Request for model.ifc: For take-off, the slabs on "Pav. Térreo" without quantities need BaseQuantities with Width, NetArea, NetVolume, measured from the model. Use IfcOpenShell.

First a look at what the model holds.

```python
import ifcopenshell
import ifcopenshell.util.element
import ifcopenshell.util.unit

model = ifcopenshell.open("model.ifc")
print(model.schema)
for unit_type in ("LENGTHUNIT", "AREAUNIT", "VOLUMEUNIT"):
    print(unit_type, ifcopenshell.util.unit.calculate_unit_scale(model, unit_type))
storey = next(s for s in model.by_type("IfcBuildingStorey") if s.Name == "Pav. Térreo")
slabs = [e for e in ifcopenshell.util.element.get_decomposition(storey) if e.is_a("IfcSlab")]
for e in sorted(slabs, key=lambda e: e.id()):
    print(e.id(), e.is_a(), e.Name, list(ifcopenshell.util.element.get_psets(e, qtos_only=True)), sep=" | ")
```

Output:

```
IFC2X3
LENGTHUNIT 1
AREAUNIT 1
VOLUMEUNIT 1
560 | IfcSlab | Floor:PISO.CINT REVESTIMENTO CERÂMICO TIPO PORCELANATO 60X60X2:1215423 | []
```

```python
import ifcopenshell
import ifcopenshell.api.pset
import ifcopenshell.geom
import ifcopenshell.util.element
import ifcopenshell.util.shape
import ifcopenshell.util.unit

model = ifcopenshell.open("model.ifc")
unit_scale = ifcopenshell.util.unit.calculate_unit_scale(model)
area_scale = ifcopenshell.util.unit.calculate_unit_scale(model, "AREAUNIT")
volume_scale = ifcopenshell.util.unit.calculate_unit_scale(model, "VOLUMEUNIT")
settings = ifcopenshell.geom.settings()

storey = next(s for s in model.by_type("IfcBuildingStorey") if s.Name == "Pav. Térreo")
slabs = [e for e in ifcopenshell.util.element.get_decomposition(storey) if e.is_a("IfcSlab")]

for e in sorted(slabs, key=lambda e: e.id()):
    if ifcopenshell.util.element.get_psets(e, qtos_only=True, should_inherit=False):
        continue
    # Geometry comes back in metres, in the element's own axes.
    shape = ifcopenshell.geom.create_shape(settings, e)
    values = {
        "Width": ifcopenshell.util.shape.get_z(shape.geometry) / unit_scale,
        "NetArea": ifcopenshell.util.shape.get_footprint_area(shape.geometry) / area_scale,
        "NetVolume": ifcopenshell.util.shape.get_volume(shape.geometry) / volume_scale,
    }
    qto = ifcopenshell.api.pset.add_qto(model, product=e, name="BaseQuantities")
    ifcopenshell.api.pset.edit_qto(model, qto=qto, properties=values)
    print(e.id(), {k: round(v, 3) for k, v in values.items()})

model.write("model_edited.ifc")
```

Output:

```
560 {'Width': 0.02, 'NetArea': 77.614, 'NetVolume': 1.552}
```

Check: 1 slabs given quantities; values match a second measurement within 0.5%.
